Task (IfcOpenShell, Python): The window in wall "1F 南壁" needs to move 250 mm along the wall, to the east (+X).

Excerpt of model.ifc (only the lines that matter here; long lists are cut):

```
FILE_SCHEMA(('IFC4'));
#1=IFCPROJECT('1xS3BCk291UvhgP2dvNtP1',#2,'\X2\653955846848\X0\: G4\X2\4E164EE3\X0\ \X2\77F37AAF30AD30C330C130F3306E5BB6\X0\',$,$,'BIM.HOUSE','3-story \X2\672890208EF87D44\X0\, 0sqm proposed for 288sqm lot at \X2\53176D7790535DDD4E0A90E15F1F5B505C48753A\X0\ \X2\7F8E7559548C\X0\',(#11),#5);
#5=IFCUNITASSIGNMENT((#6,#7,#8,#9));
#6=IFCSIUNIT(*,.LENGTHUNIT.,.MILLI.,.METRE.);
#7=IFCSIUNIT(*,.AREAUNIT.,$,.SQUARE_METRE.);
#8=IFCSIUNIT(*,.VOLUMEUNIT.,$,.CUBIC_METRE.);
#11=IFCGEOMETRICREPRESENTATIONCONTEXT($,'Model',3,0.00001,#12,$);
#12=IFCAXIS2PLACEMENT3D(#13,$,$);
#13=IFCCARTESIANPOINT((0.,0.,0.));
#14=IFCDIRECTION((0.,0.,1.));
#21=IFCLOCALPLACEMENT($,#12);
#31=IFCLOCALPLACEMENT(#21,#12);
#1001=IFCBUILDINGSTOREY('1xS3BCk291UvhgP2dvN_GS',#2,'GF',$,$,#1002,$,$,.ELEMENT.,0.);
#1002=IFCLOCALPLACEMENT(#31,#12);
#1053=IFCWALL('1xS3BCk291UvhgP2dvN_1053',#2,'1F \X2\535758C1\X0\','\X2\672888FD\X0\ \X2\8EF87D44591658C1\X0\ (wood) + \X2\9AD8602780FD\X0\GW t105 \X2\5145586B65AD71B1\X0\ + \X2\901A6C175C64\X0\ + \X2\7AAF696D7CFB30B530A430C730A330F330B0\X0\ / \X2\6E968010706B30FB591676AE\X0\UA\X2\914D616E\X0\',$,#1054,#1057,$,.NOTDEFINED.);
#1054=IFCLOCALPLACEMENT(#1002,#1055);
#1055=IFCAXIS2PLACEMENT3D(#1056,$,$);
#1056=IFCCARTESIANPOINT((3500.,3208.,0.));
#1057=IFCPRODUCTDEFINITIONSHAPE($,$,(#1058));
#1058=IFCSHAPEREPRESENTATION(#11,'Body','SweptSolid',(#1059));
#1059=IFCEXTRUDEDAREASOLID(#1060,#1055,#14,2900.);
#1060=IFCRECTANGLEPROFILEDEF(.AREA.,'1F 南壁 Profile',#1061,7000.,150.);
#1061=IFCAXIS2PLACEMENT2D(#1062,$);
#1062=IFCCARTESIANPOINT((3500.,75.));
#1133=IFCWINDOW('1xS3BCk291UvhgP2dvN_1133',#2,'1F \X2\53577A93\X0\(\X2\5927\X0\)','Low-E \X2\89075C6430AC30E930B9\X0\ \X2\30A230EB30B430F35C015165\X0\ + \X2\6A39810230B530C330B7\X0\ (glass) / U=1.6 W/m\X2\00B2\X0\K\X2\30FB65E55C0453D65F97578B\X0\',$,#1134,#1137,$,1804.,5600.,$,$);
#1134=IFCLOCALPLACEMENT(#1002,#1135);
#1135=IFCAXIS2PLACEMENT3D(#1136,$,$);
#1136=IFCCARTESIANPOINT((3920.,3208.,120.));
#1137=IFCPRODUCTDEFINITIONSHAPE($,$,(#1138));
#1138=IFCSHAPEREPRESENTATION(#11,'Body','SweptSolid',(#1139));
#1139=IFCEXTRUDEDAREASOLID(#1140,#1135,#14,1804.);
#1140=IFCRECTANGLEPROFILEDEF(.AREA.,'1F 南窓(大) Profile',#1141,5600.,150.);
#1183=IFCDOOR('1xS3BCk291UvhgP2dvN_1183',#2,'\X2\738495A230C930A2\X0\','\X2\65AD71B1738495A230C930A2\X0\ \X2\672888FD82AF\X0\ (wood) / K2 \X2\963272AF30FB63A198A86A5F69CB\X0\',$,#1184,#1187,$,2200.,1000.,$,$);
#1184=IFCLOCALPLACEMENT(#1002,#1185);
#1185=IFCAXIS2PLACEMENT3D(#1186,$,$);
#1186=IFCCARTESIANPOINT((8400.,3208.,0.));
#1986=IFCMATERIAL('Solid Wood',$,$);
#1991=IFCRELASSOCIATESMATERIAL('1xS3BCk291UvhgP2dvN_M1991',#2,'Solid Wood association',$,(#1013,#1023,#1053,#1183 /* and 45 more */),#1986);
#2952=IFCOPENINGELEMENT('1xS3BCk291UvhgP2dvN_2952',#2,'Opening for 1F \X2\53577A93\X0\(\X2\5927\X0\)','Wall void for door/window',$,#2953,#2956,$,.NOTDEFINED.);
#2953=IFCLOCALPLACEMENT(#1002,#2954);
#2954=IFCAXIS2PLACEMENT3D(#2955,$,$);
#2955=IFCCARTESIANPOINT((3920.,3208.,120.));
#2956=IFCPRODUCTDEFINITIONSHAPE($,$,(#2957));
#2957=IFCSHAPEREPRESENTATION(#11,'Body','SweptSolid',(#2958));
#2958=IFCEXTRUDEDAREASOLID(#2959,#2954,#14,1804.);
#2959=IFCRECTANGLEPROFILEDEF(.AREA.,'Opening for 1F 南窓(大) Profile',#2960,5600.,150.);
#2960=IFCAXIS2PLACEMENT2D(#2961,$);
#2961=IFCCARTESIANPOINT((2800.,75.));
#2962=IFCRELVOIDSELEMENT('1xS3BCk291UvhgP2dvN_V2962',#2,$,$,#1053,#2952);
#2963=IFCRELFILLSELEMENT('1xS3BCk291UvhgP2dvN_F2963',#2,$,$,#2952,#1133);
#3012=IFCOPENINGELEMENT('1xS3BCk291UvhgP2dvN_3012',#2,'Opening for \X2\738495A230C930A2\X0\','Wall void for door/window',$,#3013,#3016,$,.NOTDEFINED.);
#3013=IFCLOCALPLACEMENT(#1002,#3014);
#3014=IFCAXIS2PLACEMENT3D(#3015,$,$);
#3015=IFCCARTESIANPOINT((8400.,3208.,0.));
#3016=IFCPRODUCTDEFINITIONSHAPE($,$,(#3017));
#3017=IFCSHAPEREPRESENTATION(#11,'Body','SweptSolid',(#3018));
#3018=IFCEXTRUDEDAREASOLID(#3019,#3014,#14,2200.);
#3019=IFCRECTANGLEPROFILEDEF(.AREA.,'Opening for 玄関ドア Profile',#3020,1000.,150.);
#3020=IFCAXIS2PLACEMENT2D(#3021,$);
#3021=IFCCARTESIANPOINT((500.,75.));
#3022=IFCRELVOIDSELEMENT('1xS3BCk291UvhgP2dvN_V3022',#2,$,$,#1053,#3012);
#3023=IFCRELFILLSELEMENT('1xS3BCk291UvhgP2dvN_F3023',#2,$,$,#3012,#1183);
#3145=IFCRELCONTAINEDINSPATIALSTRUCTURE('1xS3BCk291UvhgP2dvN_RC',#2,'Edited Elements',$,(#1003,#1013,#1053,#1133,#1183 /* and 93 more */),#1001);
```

```python
import ifcopenshell
import ifcopenshell.api.geometry
import ifcopenshell.util.placement

model = ifcopenshell.open("model.ifc")

window = model.by_guid("1xS3BCk291UvhgP2dvN_1133")
opening = window.FillsVoids[0].RelatingOpeningElement
wall = opening.VoidsElements[0].RelatingBuildingElement

wall_matrix = ifcopenshell.util.placement.get_local_placement(wall.ObjectPlacement)
shift = wall_matrix[:3, 0] * 250.0
before = ifcopenshell.util.placement.get_local_placement(window.ObjectPlacement)[:3, 3].copy()

# The window is not placed relative to its opening, so move both.
for product in (opening, window):
    matrix = ifcopenshell.util.placement.get_local_placement(product.ObjectPlacement)
    matrix[:3, 3] += shift
    ifcopenshell.api.geometry.edit_object_placement(model, product=product, matrix=matrix, is_si=False)

after = ifcopenshell.util.placement.get_local_placement(window.ObjectPlacement)[:3, 3]
print("window moved by", (after - before).round(3) + 0.0)

model.write("model_edited.ifc")
```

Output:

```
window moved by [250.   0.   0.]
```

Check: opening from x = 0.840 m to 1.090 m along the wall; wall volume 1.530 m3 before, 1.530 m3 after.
